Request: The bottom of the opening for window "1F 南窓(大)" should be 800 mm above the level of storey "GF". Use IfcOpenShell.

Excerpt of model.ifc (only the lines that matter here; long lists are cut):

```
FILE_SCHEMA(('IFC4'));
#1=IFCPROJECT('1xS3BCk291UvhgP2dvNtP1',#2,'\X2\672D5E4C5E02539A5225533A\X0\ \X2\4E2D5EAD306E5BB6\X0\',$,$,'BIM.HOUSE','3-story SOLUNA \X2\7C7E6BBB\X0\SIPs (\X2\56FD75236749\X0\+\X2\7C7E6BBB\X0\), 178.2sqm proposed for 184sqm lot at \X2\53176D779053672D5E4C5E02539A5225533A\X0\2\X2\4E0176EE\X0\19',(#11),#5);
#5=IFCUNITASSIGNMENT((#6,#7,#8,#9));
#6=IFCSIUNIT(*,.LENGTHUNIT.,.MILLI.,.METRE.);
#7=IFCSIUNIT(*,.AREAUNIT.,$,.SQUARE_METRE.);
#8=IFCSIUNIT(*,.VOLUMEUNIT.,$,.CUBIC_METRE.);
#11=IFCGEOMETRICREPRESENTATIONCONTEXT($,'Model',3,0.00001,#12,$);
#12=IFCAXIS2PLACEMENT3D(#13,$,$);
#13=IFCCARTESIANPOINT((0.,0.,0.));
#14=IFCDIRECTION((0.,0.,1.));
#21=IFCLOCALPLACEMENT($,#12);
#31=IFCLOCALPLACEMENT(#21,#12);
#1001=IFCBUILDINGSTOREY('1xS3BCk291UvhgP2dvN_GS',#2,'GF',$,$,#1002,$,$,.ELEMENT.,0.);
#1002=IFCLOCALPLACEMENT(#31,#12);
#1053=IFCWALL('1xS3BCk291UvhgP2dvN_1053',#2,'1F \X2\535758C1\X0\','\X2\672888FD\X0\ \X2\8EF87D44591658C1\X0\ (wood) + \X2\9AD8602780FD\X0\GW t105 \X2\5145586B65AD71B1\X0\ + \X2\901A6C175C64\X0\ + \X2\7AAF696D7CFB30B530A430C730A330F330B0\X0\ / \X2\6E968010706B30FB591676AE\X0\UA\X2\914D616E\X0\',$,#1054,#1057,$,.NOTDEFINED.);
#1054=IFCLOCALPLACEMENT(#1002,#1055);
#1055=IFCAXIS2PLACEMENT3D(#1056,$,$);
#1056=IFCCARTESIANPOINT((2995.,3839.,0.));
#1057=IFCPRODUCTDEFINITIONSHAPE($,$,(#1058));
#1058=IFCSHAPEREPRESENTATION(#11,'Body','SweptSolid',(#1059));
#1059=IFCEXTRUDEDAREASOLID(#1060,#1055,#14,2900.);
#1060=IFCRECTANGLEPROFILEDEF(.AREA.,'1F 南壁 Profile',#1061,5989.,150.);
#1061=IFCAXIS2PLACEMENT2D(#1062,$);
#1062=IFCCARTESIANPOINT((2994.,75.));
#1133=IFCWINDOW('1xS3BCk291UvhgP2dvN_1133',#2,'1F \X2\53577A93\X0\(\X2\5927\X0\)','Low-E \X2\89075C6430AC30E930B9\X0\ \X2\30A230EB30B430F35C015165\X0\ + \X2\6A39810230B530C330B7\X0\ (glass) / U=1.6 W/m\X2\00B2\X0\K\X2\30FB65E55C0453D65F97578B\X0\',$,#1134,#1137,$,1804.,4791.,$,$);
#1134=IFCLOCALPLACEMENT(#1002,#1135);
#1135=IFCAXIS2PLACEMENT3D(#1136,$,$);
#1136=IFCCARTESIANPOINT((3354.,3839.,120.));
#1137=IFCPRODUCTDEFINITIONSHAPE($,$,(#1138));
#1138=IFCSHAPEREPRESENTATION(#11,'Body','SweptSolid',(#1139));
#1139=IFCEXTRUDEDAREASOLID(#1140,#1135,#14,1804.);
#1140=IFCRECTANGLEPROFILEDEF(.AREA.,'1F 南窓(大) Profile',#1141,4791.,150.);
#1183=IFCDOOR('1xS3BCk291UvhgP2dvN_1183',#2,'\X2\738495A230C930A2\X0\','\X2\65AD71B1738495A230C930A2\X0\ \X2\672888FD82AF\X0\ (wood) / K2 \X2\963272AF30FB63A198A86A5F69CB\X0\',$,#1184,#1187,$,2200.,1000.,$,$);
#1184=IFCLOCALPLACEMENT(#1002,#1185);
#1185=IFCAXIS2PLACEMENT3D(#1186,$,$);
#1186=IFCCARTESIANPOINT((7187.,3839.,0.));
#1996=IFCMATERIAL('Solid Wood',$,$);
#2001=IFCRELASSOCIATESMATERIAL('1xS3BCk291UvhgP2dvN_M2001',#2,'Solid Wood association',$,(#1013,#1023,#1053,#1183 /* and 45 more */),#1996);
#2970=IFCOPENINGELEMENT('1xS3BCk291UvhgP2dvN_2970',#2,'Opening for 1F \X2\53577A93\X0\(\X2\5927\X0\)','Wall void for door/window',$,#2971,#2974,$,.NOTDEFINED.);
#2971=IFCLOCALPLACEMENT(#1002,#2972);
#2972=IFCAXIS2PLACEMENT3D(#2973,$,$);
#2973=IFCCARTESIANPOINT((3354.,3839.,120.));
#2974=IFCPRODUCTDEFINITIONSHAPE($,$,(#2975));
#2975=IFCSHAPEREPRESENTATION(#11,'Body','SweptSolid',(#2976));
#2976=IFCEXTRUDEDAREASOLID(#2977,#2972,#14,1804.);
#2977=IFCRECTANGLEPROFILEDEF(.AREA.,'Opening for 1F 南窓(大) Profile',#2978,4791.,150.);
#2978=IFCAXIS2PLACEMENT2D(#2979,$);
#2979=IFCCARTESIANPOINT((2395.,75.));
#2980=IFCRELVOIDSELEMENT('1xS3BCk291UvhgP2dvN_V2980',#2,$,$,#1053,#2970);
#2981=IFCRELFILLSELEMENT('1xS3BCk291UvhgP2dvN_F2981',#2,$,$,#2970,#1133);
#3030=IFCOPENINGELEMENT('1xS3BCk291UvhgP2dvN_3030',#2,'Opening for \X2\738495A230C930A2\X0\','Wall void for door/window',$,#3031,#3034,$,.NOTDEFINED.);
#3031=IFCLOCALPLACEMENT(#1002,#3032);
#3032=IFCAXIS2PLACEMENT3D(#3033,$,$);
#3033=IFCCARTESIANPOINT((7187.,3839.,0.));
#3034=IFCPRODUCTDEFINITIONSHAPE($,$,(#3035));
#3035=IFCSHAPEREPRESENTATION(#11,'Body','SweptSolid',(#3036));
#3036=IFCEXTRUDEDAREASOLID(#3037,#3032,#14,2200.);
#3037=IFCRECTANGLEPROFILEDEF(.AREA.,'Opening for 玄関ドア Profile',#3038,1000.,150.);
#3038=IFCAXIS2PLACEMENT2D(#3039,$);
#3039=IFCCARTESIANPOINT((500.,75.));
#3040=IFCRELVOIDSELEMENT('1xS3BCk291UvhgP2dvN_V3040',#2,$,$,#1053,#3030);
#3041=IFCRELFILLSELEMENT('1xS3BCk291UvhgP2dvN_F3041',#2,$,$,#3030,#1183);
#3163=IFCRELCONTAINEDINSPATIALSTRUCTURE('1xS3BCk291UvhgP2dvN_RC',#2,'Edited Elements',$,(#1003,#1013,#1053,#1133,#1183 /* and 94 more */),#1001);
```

```python
import numpy as np
import ifcopenshell
import ifcopenshell.api.geometry
import ifcopenshell.geom
import ifcopenshell.util.element
import ifcopenshell.util.placement
import ifcopenshell.util.shape
import ifcopenshell.util.unit

model = ifcopenshell.open("model.ifc")
unit_scale = ifcopenshell.util.unit.calculate_unit_scale(model)

window = model.by_guid("1xS3BCk291UvhgP2dvN_1133")
opening = window.FillsVoids[0].RelatingOpeningElement
storey = ifcopenshell.util.element.get_container(window, ifc_class="IfcBuildingStorey")
level = ifcopenshell.util.placement.get_local_placement(storey.ObjectPlacement)[2, 3]

# The opening's origin need not be at the sill, so measure its lowest point.
shape = ifcopenshell.geom.create_shape(ifcopenshell.geom.settings(), opening)
bottom = ifcopenshell.util.shape.get_shape_bottom_elevation(shape, shape.geometry) / unit_scale
dz = level + 0.8 / unit_scale - bottom

shift = np.array([0.0, 0.0, dz])
# The window is not placed relative to its opening, so move both.
for product in (opening, window):
    matrix = ifcopenshell.util.placement.get_local_placement(product.ObjectPlacement)
    matrix[:3, 3] += shift
    ifcopenshell.api.geometry.edit_object_placement(model, product=product, matrix=matrix, is_si=False)

print(f"moved by {dz * unit_scale:+.3f} m")

model.write("model_v2.ifc")
```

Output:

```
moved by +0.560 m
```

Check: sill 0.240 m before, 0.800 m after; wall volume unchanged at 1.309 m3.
